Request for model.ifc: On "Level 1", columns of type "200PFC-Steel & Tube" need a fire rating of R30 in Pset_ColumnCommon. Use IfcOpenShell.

First a look at what the model holds.

```python
import ifcopenshell
import ifcopenshell.util.element

model = ifcopenshell.open("model.ifc")
print(model.schema)
storey = next(s for s in model.by_type("IfcBuildingStorey") if s.Name == "Level 1")
columns = [e for e in ifcopenshell.util.element.get_decomposition(storey) if e.is_a("IfcColumn")]
seen = {}
for e in columns:
    element_type = ifcopenshell.util.element.get_type(e)
    key = (element_type.Name if element_type != e and element_type else None, ifcopenshell.util.element.get_pset(e, "Pset_ColumnCommon", "FireRating"))
    seen[key] = seen.get(key, 0) + 1
for (name, value), count in sorted(seen.items(), key=str):
    print(count, "x", name, "|", value)
```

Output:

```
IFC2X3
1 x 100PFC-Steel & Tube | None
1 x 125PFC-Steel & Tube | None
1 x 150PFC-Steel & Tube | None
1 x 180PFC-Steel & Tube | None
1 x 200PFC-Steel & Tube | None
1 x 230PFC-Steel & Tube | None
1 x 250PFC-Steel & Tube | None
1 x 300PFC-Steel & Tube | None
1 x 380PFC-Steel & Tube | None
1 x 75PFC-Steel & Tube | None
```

```python
import ifcopenshell
import ifcopenshell.api.pset
import ifcopenshell.util.element

model = ifcopenshell.open("model.ifc")

storey = next(s for s in model.by_type("IfcBuildingStorey") if s.Name == "Level 1")
columns = [e for e in ifcopenshell.util.element.get_decomposition(storey) if e.is_a("IfcColumn")]

count = 0
for e in columns:
    element_type = ifcopenshell.util.element.get_type(e)
    if element_type in (None, e) or element_type.Name != "200PFC-Steel & Tube":
        continue
    # add_pset returns the element's existing set when there is one.
    pset = ifcopenshell.api.pset.add_pset(model, product=e, name="Pset_ColumnCommon")
    ifcopenshell.api.pset.edit_pset(model, pset=pset, properties={"FireRating": "R30"})
    count += 1

print(count, "columns updated")

model.write("model-out.ifc")
```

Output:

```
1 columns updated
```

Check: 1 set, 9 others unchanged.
